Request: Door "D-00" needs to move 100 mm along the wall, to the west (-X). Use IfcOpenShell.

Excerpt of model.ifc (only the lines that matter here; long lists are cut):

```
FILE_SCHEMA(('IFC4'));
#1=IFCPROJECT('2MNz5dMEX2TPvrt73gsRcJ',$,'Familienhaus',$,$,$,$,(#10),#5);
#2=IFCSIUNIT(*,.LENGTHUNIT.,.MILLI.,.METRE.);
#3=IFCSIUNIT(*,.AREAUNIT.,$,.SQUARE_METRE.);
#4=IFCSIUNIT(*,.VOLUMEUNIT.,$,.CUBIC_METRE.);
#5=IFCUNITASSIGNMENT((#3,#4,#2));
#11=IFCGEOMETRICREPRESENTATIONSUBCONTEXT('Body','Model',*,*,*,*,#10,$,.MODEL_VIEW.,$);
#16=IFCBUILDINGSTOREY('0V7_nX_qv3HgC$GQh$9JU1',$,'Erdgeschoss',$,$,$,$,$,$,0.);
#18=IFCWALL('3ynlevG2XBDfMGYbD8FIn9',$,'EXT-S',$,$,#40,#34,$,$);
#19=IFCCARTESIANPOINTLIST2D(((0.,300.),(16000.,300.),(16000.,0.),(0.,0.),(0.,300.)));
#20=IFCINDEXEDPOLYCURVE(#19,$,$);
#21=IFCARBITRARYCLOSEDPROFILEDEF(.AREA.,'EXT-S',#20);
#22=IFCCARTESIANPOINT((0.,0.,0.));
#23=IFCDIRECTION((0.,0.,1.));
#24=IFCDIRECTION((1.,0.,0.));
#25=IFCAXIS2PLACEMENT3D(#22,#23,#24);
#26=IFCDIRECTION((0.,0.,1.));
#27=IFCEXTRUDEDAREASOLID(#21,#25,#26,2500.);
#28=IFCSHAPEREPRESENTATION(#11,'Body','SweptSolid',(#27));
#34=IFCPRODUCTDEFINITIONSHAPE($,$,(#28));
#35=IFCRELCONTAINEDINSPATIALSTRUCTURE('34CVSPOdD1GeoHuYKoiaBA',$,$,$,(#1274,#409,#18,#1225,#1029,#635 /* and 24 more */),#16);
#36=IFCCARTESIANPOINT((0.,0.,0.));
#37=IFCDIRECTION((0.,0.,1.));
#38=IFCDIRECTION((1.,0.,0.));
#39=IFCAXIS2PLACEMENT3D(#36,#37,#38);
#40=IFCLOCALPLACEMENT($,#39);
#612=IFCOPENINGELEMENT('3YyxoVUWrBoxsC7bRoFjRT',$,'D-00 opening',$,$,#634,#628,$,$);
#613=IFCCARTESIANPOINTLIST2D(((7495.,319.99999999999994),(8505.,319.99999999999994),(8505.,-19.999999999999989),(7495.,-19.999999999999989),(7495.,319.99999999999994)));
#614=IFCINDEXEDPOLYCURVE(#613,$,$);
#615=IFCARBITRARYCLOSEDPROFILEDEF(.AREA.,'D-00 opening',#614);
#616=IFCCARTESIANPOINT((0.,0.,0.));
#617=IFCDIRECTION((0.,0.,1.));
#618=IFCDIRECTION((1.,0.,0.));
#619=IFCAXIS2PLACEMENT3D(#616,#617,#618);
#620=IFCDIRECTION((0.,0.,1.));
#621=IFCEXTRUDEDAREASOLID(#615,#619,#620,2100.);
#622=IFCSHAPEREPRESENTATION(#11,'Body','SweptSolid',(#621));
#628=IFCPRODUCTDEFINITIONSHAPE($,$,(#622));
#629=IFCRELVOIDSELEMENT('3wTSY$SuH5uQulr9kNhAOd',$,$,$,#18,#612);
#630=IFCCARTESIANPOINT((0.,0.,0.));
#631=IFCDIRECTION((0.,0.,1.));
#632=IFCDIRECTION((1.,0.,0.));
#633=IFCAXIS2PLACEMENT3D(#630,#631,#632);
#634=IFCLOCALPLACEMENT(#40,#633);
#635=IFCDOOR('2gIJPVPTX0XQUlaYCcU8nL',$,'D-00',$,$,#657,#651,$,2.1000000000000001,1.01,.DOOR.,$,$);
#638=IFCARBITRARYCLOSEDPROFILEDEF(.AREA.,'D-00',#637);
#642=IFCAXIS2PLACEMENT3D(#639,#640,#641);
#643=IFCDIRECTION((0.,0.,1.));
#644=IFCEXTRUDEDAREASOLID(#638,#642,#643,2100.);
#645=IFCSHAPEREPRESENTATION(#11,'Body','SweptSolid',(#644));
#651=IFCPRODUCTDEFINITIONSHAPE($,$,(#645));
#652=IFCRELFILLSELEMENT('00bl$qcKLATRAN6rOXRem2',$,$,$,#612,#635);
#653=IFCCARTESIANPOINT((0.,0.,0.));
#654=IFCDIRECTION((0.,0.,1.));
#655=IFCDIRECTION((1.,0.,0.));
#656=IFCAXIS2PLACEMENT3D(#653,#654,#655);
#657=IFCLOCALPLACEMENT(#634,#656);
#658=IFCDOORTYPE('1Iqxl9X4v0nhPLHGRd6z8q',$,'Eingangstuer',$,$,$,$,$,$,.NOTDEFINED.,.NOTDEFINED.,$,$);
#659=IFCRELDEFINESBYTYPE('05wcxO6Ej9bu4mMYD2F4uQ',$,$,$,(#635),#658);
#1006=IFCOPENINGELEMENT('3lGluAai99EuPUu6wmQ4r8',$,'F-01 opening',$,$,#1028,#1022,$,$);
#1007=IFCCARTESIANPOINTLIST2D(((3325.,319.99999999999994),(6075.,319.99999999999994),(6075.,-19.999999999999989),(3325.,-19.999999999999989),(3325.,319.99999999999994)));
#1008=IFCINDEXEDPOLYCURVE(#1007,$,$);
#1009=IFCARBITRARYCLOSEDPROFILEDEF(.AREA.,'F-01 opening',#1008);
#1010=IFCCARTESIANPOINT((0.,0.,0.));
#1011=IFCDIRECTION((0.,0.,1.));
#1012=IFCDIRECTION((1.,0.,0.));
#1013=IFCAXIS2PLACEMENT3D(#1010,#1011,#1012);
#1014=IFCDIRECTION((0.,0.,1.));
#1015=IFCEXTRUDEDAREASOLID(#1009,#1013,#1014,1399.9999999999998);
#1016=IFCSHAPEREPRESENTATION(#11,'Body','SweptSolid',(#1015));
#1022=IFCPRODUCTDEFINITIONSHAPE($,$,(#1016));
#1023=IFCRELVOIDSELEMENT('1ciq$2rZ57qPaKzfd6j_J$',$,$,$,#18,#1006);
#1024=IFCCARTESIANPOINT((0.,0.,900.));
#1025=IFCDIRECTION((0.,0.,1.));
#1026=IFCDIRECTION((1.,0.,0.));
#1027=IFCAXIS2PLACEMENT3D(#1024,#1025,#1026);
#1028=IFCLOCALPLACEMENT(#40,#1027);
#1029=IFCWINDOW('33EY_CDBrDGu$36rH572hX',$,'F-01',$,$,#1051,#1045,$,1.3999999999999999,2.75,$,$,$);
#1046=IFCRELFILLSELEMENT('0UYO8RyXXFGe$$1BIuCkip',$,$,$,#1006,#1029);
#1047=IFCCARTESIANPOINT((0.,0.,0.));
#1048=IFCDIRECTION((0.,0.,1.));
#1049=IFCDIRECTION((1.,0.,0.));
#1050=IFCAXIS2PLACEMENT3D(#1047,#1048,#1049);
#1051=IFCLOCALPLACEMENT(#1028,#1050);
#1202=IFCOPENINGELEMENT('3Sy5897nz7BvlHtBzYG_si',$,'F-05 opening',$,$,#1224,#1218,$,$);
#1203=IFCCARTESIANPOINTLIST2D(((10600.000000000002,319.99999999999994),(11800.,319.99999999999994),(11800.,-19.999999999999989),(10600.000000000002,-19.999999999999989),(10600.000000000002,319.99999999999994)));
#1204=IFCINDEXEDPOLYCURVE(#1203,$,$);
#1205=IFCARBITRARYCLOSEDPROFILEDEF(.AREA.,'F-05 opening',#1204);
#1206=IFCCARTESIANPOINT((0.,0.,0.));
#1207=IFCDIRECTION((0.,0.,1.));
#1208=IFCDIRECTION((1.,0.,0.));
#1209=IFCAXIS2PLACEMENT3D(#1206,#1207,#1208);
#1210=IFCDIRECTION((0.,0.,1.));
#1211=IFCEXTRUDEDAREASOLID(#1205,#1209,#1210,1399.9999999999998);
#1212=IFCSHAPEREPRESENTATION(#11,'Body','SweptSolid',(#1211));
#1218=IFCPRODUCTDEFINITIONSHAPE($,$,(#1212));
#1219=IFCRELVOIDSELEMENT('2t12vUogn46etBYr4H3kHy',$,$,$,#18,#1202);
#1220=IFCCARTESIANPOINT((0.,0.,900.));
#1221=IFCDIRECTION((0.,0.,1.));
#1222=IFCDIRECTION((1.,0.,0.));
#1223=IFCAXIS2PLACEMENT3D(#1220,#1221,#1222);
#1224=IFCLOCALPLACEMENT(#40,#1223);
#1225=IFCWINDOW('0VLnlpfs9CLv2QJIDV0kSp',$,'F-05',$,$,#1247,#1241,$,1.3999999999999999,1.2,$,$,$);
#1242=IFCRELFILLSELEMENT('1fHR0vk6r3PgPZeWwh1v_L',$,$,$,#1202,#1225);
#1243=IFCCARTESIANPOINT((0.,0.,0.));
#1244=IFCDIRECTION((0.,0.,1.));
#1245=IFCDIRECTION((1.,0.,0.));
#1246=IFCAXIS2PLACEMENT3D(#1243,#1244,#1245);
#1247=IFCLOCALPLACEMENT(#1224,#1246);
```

```python
import ifcopenshell
import ifcopenshell.api.geometry
import ifcopenshell.util.placement
import ifcopenshell.util.unit

model = ifcopenshell.open("model.ifc")
unit_scale = ifcopenshell.util.unit.calculate_unit_scale(model)

door = model.by_guid("2gIJPVPTX0XQUlaYCcU8nL")
opening = door.FillsVoids[0].RelatingOpeningElement
wall = opening.VoidsElements[0].RelatingBuildingElement

wall_matrix = ifcopenshell.util.placement.get_local_placement(wall.ObjectPlacement)
shift = wall_matrix[:3, 0] * -0.1 / unit_scale
before = ifcopenshell.util.placement.get_local_placement(door.ObjectPlacement)[:3, 3].copy()

# The door is placed relative to its opening, so it follows when the opening moves.
matrix = ifcopenshell.util.placement.get_local_placement(opening.ObjectPlacement)
matrix[:3, 3] += shift
ifcopenshell.api.geometry.edit_object_placement(
    model, product=opening, matrix=matrix, is_si=False, should_transform_children=True
)

after = ifcopenshell.util.placement.get_local_placement(door.ObjectPlacement)[:3, 3]
print("door moved by", (after - before).round(3) + 0.0)

model.write("model-out.ifc")
```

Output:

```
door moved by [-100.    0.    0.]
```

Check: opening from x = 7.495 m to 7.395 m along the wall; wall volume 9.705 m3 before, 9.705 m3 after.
